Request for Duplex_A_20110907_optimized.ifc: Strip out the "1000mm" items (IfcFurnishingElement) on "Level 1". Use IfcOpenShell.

First a look at what the model holds.

```python
import ifcopenshell
import ifcopenshell.util.element

model = ifcopenshell.open("Duplex_A_20110907_optimized.ifc")
print(model.schema)
storey = next(s for s in model.by_type("IfcBuildingStorey") if s.Name == "Level 1")
furniture = [e for e in ifcopenshell.util.element.get_decomposition(storey) if e.is_a("IfcFurnishingElement")]
seen = {}
for e in furniture:
    element_type = ifcopenshell.util.element.get_type(e)
    name = element_type.Name if element_type not in (None, e) else None
    seen[name] = seen.get(name, 0) + 1
for name, count in sorted(seen.items(), key=str):
    print(count, "x", name)
```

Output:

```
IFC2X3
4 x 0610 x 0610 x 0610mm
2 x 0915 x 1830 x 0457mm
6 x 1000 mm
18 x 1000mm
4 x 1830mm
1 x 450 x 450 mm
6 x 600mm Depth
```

```python
import ifcopenshell
import ifcopenshell.api.root
import ifcopenshell.util.element

model = ifcopenshell.open("Duplex_A_20110907_optimized.ifc")

storey = next(s for s in model.by_type("IfcBuildingStorey") if s.Name == "Level 1")
furniture = [e for e in ifcopenshell.util.element.get_decomposition(storey) if e.is_a("IfcFurnishingElement")]
targets = [e for e in furniture if (t := ifcopenshell.util.element.get_type(e)) not in (None, e) and t.Name == "1000mm"]

for e in targets:
    ifcopenshell.api.root.remove_product(model, product=e)
print(len(targets), "removed")

model.write("Duplex_A_20110907_optimized_edited.ifc")
```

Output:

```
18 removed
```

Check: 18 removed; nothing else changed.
